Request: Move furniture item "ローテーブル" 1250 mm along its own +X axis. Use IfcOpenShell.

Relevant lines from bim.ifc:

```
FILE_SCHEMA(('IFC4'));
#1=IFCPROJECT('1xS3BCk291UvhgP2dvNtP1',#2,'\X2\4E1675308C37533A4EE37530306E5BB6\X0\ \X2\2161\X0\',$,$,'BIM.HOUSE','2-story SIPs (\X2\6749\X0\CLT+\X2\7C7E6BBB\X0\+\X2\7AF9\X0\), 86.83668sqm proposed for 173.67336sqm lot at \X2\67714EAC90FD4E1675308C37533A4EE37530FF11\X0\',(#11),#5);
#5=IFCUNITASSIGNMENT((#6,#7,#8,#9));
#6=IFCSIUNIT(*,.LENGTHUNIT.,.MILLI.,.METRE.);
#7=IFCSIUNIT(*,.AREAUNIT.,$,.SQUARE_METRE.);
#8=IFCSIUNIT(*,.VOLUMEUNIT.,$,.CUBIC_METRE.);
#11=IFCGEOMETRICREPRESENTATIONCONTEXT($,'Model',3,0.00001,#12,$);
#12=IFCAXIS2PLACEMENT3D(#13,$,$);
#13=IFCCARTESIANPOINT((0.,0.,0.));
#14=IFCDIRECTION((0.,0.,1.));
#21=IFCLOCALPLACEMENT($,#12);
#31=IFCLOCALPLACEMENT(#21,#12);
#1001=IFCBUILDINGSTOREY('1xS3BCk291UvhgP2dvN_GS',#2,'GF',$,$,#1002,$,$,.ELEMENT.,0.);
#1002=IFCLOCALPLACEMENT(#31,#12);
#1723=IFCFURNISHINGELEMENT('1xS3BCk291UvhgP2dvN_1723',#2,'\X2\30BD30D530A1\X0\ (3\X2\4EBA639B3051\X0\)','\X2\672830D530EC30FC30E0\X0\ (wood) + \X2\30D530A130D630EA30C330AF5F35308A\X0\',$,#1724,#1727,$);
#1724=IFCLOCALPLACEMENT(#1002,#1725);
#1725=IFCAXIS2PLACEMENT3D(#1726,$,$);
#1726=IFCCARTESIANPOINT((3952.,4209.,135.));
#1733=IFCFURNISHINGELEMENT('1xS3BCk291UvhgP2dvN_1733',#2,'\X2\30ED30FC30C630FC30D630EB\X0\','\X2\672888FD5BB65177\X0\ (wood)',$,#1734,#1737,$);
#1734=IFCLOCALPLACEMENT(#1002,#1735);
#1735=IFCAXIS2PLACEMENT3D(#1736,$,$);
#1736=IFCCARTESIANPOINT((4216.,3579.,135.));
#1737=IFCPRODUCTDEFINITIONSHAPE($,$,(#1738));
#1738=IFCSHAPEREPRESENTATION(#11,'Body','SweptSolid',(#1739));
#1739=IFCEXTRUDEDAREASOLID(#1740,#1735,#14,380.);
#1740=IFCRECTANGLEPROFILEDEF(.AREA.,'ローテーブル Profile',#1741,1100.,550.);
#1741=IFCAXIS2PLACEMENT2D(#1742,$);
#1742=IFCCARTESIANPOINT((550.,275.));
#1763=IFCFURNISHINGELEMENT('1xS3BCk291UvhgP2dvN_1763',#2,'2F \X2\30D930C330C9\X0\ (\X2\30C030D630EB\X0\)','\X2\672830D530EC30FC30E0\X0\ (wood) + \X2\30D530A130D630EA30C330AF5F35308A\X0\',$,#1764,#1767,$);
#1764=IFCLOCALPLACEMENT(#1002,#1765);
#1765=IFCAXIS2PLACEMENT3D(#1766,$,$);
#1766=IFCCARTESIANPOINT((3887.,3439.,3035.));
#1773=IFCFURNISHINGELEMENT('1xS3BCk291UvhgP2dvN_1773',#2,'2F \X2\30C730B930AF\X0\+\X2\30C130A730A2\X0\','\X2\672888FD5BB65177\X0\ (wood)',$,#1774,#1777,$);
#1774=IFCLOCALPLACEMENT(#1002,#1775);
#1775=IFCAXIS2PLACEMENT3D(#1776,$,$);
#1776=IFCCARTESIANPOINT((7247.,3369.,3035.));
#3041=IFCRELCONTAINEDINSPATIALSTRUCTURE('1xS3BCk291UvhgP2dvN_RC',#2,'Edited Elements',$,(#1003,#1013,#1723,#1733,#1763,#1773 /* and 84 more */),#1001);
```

```python
import ifcopenshell
import ifcopenshell.api.geometry
import ifcopenshell.util.placement
import ifcopenshell.util.unit

model = ifcopenshell.open("bim.ifc")
unit_scale = ifcopenshell.util.unit.calculate_unit_scale(model)

item = model.by_guid("1xS3BCk291UvhgP2dvN_1733")
matrix = ifcopenshell.util.placement.get_local_placement(item.ObjectPlacement)
matrix[:3, 3] += matrix[:3, 0] * 1.25 / unit_scale
ifcopenshell.api.geometry.edit_object_placement(model, product=item, matrix=matrix, is_si=False)

print(ifcopenshell.util.placement.get_local_placement(item.ObjectPlacement).round(3) + 0.0)

model.write("bim_updated.ifc")
```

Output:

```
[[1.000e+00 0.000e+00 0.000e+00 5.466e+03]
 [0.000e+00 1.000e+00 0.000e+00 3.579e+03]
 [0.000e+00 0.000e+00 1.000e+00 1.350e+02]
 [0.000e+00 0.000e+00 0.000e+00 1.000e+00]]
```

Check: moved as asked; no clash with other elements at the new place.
